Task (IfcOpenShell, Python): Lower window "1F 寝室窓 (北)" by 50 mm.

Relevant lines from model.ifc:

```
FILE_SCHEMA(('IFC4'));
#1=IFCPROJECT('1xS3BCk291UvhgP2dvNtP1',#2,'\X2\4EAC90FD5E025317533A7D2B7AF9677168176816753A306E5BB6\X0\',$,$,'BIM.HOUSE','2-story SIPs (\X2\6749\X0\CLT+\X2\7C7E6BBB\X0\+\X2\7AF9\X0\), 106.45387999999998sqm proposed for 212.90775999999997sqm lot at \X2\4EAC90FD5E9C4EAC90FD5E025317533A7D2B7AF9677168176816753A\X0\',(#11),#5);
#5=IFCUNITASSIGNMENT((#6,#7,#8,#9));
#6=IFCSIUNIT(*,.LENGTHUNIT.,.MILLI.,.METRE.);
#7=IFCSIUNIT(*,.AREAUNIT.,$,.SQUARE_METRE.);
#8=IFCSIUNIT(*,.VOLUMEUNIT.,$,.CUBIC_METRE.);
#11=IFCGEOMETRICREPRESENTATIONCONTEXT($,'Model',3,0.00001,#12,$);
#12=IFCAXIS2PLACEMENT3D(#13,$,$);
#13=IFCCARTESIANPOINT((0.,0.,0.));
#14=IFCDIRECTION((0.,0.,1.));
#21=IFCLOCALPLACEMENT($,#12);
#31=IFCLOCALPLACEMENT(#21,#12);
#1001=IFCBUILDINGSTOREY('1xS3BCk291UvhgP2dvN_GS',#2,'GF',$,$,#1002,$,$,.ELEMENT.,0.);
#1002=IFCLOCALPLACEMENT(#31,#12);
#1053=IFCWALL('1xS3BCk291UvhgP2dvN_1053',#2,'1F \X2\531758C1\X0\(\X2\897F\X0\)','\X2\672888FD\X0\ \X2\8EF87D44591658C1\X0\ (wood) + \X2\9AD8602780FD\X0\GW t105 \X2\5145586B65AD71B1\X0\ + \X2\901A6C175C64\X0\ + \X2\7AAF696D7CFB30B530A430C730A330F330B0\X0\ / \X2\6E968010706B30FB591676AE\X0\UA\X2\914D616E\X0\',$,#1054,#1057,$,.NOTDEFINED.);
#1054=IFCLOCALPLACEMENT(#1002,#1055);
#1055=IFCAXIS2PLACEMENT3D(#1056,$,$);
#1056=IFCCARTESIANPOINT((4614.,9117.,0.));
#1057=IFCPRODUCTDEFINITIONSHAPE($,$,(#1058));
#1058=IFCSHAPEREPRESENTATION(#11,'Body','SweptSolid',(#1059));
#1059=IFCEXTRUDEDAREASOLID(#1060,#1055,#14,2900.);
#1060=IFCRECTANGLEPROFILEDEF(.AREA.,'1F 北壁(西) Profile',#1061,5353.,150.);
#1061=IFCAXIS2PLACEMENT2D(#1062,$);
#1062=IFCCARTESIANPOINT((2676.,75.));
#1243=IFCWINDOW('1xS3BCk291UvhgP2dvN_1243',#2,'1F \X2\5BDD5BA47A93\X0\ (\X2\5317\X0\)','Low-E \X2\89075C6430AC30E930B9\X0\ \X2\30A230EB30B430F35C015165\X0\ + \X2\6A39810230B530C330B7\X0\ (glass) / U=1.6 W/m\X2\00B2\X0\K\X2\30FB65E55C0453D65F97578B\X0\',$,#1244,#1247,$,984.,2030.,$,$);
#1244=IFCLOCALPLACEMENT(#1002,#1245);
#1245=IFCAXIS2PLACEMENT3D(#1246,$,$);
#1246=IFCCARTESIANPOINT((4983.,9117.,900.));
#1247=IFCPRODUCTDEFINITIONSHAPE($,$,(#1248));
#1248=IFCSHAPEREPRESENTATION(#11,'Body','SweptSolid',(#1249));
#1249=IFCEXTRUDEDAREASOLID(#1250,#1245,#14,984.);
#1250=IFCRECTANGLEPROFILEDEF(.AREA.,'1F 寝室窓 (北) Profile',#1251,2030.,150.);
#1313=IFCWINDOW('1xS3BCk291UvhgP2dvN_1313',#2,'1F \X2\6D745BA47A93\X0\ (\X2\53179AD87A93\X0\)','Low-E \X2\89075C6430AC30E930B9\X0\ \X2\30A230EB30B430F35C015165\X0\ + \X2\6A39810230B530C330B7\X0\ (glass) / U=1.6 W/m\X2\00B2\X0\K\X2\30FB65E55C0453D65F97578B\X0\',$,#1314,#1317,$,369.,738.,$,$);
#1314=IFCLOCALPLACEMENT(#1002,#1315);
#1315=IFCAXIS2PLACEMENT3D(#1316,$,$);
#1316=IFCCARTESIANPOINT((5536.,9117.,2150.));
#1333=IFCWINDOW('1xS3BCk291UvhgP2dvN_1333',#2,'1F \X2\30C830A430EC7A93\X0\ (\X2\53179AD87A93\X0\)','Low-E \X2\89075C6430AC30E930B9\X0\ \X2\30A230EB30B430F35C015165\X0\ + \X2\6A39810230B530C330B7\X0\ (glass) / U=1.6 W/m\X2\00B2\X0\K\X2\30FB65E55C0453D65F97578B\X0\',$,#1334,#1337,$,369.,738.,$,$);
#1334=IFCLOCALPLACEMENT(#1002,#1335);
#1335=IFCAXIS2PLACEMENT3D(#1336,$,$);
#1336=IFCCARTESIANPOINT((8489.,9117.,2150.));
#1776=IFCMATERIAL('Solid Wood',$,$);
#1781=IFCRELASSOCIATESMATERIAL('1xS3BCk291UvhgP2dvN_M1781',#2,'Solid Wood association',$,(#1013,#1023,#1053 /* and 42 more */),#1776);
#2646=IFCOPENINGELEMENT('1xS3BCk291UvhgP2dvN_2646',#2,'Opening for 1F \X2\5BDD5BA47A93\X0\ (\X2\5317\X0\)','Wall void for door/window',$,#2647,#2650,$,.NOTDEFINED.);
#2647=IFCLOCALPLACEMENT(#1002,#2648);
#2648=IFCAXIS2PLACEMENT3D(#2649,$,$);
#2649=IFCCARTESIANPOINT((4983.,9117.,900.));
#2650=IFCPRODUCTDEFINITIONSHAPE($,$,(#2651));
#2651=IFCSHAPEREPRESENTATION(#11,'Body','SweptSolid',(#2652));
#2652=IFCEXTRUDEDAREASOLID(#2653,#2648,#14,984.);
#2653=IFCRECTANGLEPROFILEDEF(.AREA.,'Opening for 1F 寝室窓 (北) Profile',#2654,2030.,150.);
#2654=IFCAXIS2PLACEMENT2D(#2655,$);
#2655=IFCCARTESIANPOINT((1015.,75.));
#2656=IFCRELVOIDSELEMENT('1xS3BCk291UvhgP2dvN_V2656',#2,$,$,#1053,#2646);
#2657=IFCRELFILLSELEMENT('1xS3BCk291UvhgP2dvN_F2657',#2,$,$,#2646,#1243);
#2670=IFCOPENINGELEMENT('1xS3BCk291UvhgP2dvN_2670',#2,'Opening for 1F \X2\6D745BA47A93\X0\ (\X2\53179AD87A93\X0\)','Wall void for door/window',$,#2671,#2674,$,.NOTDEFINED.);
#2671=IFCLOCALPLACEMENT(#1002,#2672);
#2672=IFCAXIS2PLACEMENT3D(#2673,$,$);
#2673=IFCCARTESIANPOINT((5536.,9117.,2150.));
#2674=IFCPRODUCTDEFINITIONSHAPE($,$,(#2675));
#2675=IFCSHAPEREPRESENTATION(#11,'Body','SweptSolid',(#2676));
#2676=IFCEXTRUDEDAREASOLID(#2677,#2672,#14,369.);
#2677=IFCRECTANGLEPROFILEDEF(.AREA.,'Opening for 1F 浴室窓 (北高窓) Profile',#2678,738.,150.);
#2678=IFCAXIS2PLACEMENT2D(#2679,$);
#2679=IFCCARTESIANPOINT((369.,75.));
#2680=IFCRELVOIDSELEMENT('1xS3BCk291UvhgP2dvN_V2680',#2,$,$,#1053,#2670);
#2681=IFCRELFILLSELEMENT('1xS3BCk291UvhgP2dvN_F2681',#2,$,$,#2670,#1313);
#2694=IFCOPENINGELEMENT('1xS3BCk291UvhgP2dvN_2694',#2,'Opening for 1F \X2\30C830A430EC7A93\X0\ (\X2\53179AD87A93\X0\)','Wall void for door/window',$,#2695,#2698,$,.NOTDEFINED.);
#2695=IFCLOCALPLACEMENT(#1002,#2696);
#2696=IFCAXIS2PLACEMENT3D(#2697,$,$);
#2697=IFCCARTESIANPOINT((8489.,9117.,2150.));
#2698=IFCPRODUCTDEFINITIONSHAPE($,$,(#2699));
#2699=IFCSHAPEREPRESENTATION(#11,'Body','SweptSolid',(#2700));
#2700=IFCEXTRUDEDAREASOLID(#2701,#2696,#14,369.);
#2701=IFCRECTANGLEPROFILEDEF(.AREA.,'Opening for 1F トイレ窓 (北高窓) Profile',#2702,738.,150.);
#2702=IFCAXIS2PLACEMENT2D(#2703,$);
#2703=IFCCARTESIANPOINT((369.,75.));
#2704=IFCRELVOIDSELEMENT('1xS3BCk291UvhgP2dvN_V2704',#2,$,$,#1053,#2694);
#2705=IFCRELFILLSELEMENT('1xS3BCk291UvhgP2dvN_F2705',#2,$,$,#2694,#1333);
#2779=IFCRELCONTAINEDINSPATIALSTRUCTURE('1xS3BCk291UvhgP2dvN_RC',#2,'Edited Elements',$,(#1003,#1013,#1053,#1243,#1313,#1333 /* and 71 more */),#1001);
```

```python
import numpy as np
import ifcopenshell
import ifcopenshell.api.geometry
import ifcopenshell.util.placement
import ifcopenshell.util.unit

model = ifcopenshell.open("model.ifc")
unit_scale = ifcopenshell.util.unit.calculate_unit_scale(model)

window = model.by_guid("1xS3BCk291UvhgP2dvN_1243")
opening = window.FillsVoids[0].RelatingOpeningElement
dz = -0.05 / unit_scale

shift = np.array([0.0, 0.0, dz])
# The window is not placed relative to its opening, so move both.
for product in (opening, window):
    matrix = ifcopenshell.util.placement.get_local_placement(product.ObjectPlacement)
    matrix[:3, 3] += shift
    ifcopenshell.api.geometry.edit_object_placement(model, product=product, matrix=matrix, is_si=False)

print(f"moved by {dz * unit_scale:+.3f} m")

model.write("model_edited.ifc")
```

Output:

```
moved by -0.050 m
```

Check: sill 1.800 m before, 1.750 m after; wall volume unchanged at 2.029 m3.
